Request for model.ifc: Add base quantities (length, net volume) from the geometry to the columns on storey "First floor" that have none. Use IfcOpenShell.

First a look at what the model holds.

```python
import ifcopenshell
import ifcopenshell.util.element
import ifcopenshell.util.unit

model = ifcopenshell.open("model.ifc")
print(model.schema)
for unit_type in ("LENGTHUNIT", "AREAUNIT", "VOLUMEUNIT"):
    print(unit_type, ifcopenshell.util.unit.calculate_unit_scale(model, unit_type))
storey = next(s for s in model.by_type("IfcBuildingStorey") if s.Name == "First floor")
columns = [e for e in ifcopenshell.util.element.get_decomposition(storey) if e.is_a("IfcColumn")]
for e in sorted(columns, key=lambda e: e.id()):
    print(e.id(), e.is_a(), e.Name, list(ifcopenshell.util.element.get_psets(e, qtos_only=True)), sep=" | ")
```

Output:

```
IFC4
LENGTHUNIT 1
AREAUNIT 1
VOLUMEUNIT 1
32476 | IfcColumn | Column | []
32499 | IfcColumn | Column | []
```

```python
import ifcopenshell
import ifcopenshell.api.pset
import ifcopenshell.geom
import ifcopenshell.util.element
import ifcopenshell.util.shape
import ifcopenshell.util.unit

model = ifcopenshell.open("model.ifc")
unit_scale = ifcopenshell.util.unit.calculate_unit_scale(model)
volume_scale = ifcopenshell.util.unit.calculate_unit_scale(model, "VOLUMEUNIT")
settings = ifcopenshell.geom.settings()

storey = next(s for s in model.by_type("IfcBuildingStorey") if s.Name == "First floor")
columns = [e for e in ifcopenshell.util.element.get_decomposition(storey) if e.is_a("IfcColumn")]

for e in sorted(columns, key=lambda e: e.id()):
    if ifcopenshell.util.element.get_psets(e, qtos_only=True, should_inherit=False):
        continue
    # Geometry comes back in metres, in the element's own axes.
    shape = ifcopenshell.geom.create_shape(settings, e)
    values = {
        "Length": ifcopenshell.util.shape.get_z(shape.geometry) / unit_scale,
        "NetVolume": ifcopenshell.util.shape.get_volume(shape.geometry) / volume_scale,
    }
    qto = ifcopenshell.api.pset.add_qto(model, product=e, name="Qto_ColumnBaseQuantities")
    ifcopenshell.api.pset.edit_qto(model, qto=qto, properties=values)
    print(e.id(), {k: round(v, 3) for k, v in values.items()})

model.write("model_v2.ifc")
```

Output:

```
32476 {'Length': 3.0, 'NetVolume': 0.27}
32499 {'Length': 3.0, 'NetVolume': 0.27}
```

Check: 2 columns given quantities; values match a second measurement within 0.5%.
